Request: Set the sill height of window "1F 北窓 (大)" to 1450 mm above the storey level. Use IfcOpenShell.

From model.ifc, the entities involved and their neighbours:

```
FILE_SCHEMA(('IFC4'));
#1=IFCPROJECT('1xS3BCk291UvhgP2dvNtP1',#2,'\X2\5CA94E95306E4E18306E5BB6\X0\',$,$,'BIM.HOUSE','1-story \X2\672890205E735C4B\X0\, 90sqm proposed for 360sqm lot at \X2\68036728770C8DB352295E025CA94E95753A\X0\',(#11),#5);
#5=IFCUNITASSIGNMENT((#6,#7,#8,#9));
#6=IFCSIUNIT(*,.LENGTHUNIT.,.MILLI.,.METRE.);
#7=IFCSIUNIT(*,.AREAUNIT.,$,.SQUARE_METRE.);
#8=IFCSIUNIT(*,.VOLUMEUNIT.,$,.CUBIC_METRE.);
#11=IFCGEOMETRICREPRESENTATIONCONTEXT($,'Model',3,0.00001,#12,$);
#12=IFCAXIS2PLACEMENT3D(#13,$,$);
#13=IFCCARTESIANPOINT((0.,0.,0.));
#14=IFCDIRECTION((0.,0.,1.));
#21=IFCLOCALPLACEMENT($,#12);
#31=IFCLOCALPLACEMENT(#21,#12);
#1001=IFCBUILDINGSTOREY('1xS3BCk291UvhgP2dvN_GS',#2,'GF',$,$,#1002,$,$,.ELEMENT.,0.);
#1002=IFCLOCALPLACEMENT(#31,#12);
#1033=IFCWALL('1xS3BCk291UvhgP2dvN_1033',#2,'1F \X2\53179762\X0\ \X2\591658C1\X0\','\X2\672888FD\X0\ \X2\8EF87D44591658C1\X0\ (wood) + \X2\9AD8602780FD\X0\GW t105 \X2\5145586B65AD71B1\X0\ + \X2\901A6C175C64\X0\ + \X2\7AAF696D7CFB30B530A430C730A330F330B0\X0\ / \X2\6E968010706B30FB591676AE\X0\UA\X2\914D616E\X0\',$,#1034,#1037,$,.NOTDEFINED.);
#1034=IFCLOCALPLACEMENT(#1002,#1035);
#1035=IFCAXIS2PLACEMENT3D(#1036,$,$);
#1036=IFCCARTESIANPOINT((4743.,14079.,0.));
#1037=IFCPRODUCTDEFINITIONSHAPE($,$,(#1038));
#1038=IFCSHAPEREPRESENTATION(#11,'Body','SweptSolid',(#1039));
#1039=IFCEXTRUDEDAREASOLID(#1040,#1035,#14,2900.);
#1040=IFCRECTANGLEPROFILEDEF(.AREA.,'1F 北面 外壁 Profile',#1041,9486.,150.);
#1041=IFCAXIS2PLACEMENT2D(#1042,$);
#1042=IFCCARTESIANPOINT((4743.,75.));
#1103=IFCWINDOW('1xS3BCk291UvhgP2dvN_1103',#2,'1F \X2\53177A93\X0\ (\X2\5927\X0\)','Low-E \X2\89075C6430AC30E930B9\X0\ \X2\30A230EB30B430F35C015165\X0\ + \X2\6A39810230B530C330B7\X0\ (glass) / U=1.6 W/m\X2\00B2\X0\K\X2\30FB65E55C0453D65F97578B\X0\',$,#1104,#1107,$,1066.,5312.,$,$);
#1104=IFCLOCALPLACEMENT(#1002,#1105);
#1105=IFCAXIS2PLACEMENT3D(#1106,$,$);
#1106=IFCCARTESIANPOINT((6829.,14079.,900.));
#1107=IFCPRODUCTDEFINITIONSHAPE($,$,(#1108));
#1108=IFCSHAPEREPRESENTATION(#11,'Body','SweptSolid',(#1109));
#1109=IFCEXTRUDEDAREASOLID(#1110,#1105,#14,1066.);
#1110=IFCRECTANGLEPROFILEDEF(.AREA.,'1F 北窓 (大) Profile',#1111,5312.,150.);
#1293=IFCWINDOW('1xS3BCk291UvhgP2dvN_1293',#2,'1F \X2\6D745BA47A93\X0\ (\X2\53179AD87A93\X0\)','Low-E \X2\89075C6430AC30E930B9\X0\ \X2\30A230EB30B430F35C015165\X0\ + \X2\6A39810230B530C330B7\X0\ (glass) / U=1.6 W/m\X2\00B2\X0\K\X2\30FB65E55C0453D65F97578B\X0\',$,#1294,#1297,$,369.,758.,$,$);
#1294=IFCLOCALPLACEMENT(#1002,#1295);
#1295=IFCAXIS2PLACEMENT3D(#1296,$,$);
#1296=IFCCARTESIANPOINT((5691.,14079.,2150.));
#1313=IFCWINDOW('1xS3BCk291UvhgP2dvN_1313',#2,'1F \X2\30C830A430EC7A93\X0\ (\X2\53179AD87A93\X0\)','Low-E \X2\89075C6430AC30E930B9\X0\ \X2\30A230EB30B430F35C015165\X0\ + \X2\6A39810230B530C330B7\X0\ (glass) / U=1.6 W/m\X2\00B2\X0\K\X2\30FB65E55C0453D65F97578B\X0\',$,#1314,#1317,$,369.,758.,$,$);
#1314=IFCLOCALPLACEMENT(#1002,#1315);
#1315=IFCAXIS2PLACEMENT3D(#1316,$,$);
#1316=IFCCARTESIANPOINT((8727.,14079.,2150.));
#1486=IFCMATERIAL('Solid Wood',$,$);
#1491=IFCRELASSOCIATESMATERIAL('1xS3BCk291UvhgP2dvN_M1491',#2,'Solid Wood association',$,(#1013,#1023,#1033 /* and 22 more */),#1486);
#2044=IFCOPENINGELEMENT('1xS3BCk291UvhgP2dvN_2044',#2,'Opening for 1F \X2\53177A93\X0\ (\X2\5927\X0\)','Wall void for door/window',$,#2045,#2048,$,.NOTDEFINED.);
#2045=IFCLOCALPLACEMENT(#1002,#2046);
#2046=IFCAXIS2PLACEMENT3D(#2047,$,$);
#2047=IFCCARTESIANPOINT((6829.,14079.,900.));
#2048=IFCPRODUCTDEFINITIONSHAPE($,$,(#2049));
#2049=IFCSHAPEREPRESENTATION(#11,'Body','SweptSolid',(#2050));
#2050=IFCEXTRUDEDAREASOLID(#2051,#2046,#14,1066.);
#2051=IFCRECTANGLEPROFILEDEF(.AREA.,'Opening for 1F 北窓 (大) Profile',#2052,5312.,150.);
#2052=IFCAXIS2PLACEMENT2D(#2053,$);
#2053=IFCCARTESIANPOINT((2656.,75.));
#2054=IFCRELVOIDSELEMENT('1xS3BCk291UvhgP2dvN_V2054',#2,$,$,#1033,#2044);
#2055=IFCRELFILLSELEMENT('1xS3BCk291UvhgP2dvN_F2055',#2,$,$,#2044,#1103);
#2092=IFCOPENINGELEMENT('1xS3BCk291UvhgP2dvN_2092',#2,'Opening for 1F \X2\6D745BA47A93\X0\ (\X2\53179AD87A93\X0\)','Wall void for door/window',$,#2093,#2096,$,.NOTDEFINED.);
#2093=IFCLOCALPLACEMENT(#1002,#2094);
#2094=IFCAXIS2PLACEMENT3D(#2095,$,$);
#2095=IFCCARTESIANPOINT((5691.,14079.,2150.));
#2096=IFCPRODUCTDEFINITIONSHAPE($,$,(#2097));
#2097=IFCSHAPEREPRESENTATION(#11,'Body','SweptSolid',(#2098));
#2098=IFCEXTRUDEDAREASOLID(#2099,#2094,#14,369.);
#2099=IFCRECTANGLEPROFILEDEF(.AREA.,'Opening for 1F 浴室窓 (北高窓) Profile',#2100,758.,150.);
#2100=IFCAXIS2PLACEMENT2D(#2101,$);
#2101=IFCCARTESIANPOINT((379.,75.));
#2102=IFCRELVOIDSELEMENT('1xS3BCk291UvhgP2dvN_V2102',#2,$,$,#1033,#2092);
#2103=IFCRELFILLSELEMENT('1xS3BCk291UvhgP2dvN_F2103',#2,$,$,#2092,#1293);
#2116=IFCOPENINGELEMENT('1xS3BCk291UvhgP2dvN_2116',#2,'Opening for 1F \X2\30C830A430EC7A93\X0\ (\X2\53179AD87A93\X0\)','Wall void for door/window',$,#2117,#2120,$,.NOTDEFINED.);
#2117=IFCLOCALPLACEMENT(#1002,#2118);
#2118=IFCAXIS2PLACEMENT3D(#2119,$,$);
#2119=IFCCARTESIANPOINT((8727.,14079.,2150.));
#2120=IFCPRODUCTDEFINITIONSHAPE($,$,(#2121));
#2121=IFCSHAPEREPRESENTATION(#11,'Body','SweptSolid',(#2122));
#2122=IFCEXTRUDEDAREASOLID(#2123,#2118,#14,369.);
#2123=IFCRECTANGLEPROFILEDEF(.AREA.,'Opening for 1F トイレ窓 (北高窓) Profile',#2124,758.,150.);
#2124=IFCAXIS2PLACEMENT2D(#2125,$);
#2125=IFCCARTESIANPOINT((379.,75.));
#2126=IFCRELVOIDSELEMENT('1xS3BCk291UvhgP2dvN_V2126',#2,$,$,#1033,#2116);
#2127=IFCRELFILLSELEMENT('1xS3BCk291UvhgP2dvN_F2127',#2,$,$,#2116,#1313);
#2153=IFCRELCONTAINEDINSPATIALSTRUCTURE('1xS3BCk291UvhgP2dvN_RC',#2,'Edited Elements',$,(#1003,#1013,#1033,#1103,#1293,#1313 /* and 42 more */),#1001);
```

```python
import numpy as np
import ifcopenshell
import ifcopenshell.api.geometry
import ifcopenshell.geom
import ifcopenshell.util.element
import ifcopenshell.util.placement
import ifcopenshell.util.shape
import ifcopenshell.util.unit

model = ifcopenshell.open("model.ifc")
unit_scale = ifcopenshell.util.unit.calculate_unit_scale(model)

window = model.by_guid("1xS3BCk291UvhgP2dvN_1103")
opening = window.FillsVoids[0].RelatingOpeningElement
storey = ifcopenshell.util.element.get_container(window, ifc_class="IfcBuildingStorey")
level = ifcopenshell.util.placement.get_local_placement(storey.ObjectPlacement)[2, 3]

# The opening's origin need not be at the sill, so measure its lowest point.
shape = ifcopenshell.geom.create_shape(ifcopenshell.geom.settings(), opening)
bottom = ifcopenshell.util.shape.get_shape_bottom_elevation(shape, shape.geometry) / unit_scale
dz = level + 1.45 / unit_scale - bottom

shift = np.array([0.0, 0.0, dz])
# The window is not placed relative to its opening, so move both.
for product in (opening, window):
    matrix = ifcopenshell.util.placement.get_local_placement(product.ObjectPlacement)
    matrix[:3, 3] += shift
    ifcopenshell.api.geometry.edit_object_placement(model, product=product, matrix=matrix, is_si=False)

print(f"moved by {dz * unit_scale:+.3f} m")

model.write("model_rev.ifc")
```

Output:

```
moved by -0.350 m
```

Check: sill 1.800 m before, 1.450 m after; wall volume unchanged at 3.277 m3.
